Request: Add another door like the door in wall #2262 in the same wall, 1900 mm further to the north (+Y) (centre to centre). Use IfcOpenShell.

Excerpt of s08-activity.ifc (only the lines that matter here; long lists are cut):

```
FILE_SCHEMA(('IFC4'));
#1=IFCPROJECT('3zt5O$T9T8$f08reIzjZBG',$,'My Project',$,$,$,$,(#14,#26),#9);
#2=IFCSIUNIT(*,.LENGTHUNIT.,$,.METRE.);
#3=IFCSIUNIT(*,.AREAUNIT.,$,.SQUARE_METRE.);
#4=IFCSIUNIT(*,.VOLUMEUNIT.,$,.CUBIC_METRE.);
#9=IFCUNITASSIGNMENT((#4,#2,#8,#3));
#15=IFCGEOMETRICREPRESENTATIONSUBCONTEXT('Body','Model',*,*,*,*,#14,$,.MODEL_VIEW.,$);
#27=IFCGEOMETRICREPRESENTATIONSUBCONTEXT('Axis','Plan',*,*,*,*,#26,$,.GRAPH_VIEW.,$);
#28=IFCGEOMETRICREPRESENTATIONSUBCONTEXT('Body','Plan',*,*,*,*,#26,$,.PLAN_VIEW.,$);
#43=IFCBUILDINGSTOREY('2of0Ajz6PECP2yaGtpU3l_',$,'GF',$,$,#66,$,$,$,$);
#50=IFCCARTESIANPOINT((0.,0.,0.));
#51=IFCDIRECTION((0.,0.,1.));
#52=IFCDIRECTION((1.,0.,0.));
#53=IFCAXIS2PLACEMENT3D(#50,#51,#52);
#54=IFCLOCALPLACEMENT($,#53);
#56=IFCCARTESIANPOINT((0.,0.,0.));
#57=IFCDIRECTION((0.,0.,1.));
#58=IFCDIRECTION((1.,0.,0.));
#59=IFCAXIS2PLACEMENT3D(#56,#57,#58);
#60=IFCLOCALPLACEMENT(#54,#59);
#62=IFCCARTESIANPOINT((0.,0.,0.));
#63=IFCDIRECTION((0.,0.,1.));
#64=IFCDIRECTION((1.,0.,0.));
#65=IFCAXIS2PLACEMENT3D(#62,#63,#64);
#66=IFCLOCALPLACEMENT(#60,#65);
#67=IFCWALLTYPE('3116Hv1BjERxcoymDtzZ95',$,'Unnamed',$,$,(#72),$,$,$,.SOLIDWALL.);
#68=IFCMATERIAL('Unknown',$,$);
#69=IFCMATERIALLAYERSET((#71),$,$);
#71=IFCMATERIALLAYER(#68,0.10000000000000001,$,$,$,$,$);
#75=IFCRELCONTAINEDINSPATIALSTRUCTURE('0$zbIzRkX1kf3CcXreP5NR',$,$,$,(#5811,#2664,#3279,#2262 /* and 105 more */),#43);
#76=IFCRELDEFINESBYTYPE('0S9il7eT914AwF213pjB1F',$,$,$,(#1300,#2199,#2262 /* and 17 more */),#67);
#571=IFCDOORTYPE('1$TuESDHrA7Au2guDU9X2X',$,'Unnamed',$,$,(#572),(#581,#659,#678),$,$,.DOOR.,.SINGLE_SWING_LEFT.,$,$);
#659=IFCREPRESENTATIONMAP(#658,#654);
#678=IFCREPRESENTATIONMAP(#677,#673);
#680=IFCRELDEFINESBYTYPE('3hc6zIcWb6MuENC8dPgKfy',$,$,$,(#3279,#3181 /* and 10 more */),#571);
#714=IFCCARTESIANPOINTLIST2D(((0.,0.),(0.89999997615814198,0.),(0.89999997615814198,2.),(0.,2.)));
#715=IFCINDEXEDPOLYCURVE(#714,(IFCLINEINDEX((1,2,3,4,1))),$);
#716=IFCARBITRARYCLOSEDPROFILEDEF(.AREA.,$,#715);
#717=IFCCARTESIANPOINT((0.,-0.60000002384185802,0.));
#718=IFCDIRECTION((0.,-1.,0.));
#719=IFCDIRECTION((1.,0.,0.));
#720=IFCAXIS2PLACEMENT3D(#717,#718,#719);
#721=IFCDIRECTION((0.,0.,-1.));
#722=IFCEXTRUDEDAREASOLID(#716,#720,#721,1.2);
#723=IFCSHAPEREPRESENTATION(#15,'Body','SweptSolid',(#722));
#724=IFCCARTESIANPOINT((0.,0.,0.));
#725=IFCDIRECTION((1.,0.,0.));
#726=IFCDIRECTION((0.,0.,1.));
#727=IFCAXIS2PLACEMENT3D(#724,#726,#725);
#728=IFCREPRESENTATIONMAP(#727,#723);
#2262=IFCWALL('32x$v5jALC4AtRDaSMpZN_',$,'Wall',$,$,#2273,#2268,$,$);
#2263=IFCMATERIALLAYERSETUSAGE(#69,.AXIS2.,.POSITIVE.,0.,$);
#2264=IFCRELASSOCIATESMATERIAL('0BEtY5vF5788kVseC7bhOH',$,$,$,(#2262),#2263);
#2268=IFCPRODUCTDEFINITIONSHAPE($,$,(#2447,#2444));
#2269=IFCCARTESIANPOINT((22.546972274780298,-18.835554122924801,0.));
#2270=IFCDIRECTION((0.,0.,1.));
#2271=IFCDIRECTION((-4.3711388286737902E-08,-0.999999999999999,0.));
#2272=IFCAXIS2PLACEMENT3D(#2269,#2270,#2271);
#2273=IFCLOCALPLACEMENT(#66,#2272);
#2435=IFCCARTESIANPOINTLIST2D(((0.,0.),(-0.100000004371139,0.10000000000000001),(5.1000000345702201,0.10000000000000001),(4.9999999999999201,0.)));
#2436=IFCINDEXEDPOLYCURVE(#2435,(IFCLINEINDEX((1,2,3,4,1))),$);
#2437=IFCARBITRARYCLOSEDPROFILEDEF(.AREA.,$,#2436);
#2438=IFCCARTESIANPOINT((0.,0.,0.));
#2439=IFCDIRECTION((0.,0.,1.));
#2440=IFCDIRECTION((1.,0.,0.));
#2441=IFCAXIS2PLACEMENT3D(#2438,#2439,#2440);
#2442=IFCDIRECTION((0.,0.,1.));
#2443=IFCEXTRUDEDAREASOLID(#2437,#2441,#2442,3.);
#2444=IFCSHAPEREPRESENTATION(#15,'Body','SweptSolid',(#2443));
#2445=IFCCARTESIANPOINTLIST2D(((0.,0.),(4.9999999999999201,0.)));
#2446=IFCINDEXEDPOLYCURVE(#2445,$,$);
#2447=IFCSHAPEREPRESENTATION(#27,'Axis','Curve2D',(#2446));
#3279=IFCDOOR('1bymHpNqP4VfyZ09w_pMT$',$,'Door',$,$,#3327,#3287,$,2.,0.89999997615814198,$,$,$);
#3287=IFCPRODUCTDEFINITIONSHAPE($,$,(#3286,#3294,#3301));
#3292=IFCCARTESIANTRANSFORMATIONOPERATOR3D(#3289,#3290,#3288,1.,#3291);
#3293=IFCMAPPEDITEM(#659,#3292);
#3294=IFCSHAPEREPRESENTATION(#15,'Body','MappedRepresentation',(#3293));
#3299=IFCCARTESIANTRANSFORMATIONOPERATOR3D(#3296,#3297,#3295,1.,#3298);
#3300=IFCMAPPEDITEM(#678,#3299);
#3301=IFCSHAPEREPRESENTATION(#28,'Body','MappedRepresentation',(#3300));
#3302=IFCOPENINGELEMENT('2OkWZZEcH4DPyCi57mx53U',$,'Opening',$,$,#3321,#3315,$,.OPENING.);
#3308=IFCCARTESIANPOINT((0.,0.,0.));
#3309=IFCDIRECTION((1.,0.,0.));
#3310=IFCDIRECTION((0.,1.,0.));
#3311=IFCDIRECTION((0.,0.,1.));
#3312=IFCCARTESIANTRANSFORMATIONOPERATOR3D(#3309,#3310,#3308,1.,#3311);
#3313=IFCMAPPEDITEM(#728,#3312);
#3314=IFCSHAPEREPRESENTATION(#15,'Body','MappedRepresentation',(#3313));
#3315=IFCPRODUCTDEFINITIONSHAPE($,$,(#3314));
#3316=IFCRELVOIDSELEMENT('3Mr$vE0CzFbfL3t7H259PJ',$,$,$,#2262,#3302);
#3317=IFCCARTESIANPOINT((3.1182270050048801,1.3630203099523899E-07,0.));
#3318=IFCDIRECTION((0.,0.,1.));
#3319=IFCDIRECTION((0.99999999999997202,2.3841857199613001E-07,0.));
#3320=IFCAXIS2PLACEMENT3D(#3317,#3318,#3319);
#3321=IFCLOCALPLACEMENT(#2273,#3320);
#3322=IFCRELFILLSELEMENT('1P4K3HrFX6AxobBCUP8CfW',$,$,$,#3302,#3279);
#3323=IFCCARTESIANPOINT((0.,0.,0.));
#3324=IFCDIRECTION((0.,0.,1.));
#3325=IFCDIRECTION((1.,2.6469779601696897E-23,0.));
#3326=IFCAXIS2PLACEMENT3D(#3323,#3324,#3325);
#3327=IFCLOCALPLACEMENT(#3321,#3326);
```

```python
import ifcopenshell
import ifcopenshell.api.feature
import ifcopenshell.api.geometry
import ifcopenshell.api.root
import ifcopenshell.geom
import ifcopenshell.util.element
import ifcopenshell.util.placement
import ifcopenshell.util.shape
import ifcopenshell.util.unit

model = ifcopenshell.open("s08-activity.ifc")
unit_scale = ifcopenshell.util.unit.calculate_unit_scale(model)
settings = ifcopenshell.geom.settings()


def volume(element):
    """Net volume in cubic metres, openings subtracted."""
    shape = ifcopenshell.geom.create_shape(settings, element)
    return ifcopenshell.util.shape.get_volume(shape.geometry)


door = model.by_guid("1bymHpNqP4VfyZ09w_pMT$")
opening = door.FillsVoids[0].RelatingOpeningElement
wall = opening.VoidsElements[0].RelatingBuildingElement
before = volume(wall)
shift = ifcopenshell.util.placement.get_local_placement(wall.ObjectPlacement)[:3, 0] * -1.9 / unit_scale

# copy_class copies the void relationship, type, container and properties, but no geometry.
new_opening = ifcopenshell.api.root.copy_class(model, product=opening)
new_opening.Representation = ifcopenshell.util.element.copy_deep(
    model, opening.Representation, exclude=["IfcGeometricRepresentationContext", "IfcRepresentationMap"]
)
new_door = ifcopenshell.api.root.copy_class(model, product=door)
new_door.Representation = ifcopenshell.util.element.copy_deep(
    model, door.Representation, exclude=["IfcGeometricRepresentationContext", "IfcRepresentationMap"]
)
ifcopenshell.api.feature.add_filling(model, opening=new_opening, element=new_door)

for old, new in ((opening, new_opening), (door, new_door)):
    matrix = ifcopenshell.util.placement.get_local_placement(old.ObjectPlacement)
    matrix[:3, 3] += shift
    ifcopenshell.api.geometry.edit_object_placement(model, product=new, matrix=matrix, is_si=False)

after = volume(wall)

print(f"wall volume {before:.3f} -> {after:.3f} m3")

model.write("s08-activity_v2.ifc")
```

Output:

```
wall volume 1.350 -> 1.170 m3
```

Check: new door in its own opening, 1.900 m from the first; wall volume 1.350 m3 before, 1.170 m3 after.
